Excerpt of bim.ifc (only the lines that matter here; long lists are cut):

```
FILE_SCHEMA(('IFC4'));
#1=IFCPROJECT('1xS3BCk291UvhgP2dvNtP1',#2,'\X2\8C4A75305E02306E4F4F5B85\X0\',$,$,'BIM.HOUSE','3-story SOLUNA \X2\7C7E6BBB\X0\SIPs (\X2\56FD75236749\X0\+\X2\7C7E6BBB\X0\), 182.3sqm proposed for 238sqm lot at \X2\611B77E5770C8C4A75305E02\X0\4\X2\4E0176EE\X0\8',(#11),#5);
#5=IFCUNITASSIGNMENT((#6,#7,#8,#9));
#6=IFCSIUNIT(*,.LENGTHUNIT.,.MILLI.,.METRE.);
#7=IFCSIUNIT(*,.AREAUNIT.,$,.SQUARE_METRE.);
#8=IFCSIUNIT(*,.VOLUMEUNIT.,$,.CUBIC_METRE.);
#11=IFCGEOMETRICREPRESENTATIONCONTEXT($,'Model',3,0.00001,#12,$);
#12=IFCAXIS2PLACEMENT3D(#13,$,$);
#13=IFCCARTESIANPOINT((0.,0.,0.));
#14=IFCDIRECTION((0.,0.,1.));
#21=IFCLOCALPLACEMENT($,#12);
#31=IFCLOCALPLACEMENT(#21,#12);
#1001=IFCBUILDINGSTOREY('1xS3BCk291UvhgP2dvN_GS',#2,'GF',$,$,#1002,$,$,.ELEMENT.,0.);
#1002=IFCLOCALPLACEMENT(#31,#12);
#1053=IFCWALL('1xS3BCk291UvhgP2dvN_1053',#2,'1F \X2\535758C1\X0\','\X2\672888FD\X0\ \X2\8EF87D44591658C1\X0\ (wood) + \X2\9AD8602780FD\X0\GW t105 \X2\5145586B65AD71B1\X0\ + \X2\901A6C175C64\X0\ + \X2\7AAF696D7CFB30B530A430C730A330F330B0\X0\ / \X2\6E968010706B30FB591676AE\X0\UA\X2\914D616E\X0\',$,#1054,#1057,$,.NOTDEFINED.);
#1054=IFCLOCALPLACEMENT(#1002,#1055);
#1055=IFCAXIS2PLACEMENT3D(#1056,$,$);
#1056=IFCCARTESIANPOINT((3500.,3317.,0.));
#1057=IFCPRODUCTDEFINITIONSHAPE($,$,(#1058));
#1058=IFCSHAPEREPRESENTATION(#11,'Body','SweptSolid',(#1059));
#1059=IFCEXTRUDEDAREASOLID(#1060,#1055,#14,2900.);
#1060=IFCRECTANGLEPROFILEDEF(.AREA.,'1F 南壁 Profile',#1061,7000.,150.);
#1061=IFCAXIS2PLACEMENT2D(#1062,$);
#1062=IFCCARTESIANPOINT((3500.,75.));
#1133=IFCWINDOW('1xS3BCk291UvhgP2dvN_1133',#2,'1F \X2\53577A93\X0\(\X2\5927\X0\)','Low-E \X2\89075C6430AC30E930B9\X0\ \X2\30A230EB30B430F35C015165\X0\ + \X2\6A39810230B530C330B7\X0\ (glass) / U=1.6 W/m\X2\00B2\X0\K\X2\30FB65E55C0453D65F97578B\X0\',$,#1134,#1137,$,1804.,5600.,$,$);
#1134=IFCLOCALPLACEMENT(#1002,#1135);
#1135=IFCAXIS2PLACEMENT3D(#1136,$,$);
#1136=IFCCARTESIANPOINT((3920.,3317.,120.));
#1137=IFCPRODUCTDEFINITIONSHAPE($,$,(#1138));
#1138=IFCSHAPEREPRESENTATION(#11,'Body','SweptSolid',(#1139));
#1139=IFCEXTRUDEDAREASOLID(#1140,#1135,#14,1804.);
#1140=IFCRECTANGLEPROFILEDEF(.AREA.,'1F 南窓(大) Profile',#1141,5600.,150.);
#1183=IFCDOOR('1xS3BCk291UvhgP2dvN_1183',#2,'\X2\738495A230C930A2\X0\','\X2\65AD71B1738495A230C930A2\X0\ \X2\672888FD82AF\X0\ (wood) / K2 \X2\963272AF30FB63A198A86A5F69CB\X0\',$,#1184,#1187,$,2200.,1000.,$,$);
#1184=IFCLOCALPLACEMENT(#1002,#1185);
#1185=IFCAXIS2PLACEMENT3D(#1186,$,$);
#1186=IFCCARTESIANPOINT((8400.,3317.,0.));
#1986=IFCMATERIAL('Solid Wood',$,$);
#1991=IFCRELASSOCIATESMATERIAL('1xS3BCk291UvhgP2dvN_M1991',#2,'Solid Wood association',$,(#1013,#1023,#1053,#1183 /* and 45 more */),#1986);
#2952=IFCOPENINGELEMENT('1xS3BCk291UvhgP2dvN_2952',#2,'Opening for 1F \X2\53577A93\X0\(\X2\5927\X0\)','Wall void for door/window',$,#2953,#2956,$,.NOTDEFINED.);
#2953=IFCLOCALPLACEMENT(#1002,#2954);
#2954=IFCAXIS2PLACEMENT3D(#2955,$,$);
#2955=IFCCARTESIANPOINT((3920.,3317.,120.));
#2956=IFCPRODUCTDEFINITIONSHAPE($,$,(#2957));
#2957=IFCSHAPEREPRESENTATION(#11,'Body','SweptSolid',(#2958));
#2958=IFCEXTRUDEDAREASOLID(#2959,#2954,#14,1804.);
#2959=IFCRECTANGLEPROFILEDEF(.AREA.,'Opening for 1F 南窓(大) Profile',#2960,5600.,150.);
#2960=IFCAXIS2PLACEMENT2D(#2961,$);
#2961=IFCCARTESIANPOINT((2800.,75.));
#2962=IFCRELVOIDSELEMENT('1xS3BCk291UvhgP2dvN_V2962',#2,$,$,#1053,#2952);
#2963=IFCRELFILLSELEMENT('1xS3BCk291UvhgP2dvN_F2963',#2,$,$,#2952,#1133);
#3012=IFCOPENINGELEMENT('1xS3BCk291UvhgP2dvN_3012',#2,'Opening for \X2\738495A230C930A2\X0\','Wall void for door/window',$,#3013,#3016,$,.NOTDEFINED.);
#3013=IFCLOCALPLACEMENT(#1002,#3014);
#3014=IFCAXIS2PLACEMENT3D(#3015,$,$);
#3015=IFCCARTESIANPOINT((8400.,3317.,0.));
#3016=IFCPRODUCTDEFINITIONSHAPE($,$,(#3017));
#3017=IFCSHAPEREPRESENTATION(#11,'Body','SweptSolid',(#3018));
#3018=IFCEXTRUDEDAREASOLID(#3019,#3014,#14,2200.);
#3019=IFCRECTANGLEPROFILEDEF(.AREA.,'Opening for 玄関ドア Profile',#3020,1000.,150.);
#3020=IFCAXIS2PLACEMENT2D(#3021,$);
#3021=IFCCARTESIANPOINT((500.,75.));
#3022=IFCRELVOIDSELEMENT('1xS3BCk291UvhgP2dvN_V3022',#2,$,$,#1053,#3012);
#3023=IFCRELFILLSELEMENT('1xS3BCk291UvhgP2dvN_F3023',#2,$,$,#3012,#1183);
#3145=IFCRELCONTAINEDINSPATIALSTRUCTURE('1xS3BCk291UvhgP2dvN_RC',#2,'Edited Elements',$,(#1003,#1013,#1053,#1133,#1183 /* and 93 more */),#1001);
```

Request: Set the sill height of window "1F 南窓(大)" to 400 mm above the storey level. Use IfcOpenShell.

```python
import numpy as np
import ifcopenshell
import ifcopenshell.api.geometry
import ifcopenshell.geom
import ifcopenshell.util.element
import ifcopenshell.util.placement
import ifcopenshell.util.shape
import ifcopenshell.util.unit

model = ifcopenshell.open("bim.ifc")
unit_scale = ifcopenshell.util.unit.calculate_unit_scale(model)

window = model.by_guid("1xS3BCk291UvhgP2dvN_1133")
opening = window.FillsVoids[0].RelatingOpeningElement
storey = ifcopenshell.util.element.get_container(window, ifc_class="IfcBuildingStorey")
level = ifcopenshell.util.placement.get_local_placement(storey.ObjectPlacement)[2, 3]

# The opening's origin need not be at the sill, so measure its lowest point.
shape = ifcopenshell.geom.create_shape(ifcopenshell.geom.settings(), opening)
bottom = ifcopenshell.util.shape.get_shape_bottom_elevation(shape, shape.geometry) / unit_scale
dz = level + 0.4 / unit_scale - bottom

shift = np.array([0.0, 0.0, dz])
# The window is not placed relative to its opening, so move both.
for product in (opening, window):
    matrix = ifcopenshell.util.placement.get_local_placement(product.ObjectPlacement)
    matrix[:3, 3] += shift
    ifcopenshell.api.geometry.edit_object_placement(model, product=product, matrix=matrix, is_si=False)

print(f"moved by {dz * unit_scale:+.3f} m")

model.write("bim_edited.ifc")
```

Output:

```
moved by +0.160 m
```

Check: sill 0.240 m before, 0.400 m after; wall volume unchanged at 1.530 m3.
